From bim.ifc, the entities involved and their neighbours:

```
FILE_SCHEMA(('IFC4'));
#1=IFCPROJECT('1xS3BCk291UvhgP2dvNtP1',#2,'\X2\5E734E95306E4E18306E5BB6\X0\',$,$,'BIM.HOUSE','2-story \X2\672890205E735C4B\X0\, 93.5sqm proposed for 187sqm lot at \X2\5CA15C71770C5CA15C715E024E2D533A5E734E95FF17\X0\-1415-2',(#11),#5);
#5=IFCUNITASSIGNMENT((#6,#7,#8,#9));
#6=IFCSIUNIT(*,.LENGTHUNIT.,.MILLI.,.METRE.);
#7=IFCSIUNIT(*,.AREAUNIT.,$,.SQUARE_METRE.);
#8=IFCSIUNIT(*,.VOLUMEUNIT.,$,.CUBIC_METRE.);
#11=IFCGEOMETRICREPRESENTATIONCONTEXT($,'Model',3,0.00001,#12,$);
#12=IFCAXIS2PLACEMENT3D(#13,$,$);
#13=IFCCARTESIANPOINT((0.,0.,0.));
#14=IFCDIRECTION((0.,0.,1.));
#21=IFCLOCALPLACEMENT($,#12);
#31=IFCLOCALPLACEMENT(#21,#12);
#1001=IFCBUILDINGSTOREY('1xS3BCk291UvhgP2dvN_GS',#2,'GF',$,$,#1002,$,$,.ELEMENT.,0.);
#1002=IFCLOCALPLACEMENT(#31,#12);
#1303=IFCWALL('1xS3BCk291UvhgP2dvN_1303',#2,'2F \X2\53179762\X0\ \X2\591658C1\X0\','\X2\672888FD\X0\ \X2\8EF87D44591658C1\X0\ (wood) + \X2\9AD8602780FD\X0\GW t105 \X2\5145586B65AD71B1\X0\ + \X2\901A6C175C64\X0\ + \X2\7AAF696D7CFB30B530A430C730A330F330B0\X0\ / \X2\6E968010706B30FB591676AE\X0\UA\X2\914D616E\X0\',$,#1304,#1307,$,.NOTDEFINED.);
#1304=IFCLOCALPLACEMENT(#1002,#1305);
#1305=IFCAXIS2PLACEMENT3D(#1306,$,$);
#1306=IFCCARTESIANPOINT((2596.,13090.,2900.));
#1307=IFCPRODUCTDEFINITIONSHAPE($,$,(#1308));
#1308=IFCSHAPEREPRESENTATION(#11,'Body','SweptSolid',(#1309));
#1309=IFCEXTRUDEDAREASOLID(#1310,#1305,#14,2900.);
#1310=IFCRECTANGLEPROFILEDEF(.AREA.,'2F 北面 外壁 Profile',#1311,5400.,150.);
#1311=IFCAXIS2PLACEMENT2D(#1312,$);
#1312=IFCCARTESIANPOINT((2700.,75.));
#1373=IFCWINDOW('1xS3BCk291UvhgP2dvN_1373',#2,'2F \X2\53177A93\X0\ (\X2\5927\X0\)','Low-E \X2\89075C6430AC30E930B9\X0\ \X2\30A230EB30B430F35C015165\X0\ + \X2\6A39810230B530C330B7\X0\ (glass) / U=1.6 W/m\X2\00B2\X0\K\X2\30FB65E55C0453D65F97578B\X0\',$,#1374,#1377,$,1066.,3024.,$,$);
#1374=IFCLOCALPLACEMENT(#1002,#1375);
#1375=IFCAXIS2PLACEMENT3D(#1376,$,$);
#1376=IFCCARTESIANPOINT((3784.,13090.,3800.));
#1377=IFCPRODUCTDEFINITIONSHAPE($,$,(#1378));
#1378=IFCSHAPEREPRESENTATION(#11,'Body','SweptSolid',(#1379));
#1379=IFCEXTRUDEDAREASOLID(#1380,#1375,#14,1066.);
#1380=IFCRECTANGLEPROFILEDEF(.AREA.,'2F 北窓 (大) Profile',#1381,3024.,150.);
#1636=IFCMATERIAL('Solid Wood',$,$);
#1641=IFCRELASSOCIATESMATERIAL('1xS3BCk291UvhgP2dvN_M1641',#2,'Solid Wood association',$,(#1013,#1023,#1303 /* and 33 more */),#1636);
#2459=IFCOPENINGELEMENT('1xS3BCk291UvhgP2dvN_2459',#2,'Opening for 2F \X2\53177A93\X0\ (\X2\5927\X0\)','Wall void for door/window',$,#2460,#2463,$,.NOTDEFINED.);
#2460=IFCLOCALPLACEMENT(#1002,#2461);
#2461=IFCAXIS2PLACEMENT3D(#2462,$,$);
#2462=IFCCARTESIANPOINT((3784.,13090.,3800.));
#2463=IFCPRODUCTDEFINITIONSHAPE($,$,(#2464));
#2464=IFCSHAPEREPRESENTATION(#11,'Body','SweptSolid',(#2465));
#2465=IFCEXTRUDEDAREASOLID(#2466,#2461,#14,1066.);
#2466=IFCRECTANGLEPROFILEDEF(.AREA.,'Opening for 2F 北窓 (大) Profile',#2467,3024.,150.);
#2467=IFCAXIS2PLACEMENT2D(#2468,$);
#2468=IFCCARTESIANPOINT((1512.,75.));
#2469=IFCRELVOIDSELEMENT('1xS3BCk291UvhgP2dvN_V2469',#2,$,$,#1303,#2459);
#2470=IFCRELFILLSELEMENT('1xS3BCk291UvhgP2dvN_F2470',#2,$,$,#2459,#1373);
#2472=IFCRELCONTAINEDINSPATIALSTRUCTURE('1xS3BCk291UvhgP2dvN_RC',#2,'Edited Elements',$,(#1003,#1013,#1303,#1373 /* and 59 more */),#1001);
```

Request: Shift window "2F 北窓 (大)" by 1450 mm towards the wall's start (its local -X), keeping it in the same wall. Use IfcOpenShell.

```python
import ifcopenshell
import ifcopenshell.api.geometry
import ifcopenshell.util.placement

model = ifcopenshell.open("bim.ifc")

window = model.by_id(1373)
opening = window.FillsVoids[0].RelatingOpeningElement
wall = opening.VoidsElements[0].RelatingBuildingElement

wall_matrix = ifcopenshell.util.placement.get_local_placement(wall.ObjectPlacement)
shift = wall_matrix[:3, 0] * -1450.0
before = ifcopenshell.util.placement.get_local_placement(window.ObjectPlacement)[:3, 3].copy()

# The window is not placed relative to its opening, so move both.
for product in (opening, window):
    matrix = ifcopenshell.util.placement.get_local_placement(product.ObjectPlacement)
    matrix[:3, 3] += shift
    ifcopenshell.api.geometry.edit_object_placement(model, product=product, matrix=matrix, is_si=False)

after = ifcopenshell.util.placement.get_local_placement(window.ObjectPlacement)[:3, 3]
print("window moved by", (after - before).round(3) + 0.0)

model.write("bim-out.ifc")
```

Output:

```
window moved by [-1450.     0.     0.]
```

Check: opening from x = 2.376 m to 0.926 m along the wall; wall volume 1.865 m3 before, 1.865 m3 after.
